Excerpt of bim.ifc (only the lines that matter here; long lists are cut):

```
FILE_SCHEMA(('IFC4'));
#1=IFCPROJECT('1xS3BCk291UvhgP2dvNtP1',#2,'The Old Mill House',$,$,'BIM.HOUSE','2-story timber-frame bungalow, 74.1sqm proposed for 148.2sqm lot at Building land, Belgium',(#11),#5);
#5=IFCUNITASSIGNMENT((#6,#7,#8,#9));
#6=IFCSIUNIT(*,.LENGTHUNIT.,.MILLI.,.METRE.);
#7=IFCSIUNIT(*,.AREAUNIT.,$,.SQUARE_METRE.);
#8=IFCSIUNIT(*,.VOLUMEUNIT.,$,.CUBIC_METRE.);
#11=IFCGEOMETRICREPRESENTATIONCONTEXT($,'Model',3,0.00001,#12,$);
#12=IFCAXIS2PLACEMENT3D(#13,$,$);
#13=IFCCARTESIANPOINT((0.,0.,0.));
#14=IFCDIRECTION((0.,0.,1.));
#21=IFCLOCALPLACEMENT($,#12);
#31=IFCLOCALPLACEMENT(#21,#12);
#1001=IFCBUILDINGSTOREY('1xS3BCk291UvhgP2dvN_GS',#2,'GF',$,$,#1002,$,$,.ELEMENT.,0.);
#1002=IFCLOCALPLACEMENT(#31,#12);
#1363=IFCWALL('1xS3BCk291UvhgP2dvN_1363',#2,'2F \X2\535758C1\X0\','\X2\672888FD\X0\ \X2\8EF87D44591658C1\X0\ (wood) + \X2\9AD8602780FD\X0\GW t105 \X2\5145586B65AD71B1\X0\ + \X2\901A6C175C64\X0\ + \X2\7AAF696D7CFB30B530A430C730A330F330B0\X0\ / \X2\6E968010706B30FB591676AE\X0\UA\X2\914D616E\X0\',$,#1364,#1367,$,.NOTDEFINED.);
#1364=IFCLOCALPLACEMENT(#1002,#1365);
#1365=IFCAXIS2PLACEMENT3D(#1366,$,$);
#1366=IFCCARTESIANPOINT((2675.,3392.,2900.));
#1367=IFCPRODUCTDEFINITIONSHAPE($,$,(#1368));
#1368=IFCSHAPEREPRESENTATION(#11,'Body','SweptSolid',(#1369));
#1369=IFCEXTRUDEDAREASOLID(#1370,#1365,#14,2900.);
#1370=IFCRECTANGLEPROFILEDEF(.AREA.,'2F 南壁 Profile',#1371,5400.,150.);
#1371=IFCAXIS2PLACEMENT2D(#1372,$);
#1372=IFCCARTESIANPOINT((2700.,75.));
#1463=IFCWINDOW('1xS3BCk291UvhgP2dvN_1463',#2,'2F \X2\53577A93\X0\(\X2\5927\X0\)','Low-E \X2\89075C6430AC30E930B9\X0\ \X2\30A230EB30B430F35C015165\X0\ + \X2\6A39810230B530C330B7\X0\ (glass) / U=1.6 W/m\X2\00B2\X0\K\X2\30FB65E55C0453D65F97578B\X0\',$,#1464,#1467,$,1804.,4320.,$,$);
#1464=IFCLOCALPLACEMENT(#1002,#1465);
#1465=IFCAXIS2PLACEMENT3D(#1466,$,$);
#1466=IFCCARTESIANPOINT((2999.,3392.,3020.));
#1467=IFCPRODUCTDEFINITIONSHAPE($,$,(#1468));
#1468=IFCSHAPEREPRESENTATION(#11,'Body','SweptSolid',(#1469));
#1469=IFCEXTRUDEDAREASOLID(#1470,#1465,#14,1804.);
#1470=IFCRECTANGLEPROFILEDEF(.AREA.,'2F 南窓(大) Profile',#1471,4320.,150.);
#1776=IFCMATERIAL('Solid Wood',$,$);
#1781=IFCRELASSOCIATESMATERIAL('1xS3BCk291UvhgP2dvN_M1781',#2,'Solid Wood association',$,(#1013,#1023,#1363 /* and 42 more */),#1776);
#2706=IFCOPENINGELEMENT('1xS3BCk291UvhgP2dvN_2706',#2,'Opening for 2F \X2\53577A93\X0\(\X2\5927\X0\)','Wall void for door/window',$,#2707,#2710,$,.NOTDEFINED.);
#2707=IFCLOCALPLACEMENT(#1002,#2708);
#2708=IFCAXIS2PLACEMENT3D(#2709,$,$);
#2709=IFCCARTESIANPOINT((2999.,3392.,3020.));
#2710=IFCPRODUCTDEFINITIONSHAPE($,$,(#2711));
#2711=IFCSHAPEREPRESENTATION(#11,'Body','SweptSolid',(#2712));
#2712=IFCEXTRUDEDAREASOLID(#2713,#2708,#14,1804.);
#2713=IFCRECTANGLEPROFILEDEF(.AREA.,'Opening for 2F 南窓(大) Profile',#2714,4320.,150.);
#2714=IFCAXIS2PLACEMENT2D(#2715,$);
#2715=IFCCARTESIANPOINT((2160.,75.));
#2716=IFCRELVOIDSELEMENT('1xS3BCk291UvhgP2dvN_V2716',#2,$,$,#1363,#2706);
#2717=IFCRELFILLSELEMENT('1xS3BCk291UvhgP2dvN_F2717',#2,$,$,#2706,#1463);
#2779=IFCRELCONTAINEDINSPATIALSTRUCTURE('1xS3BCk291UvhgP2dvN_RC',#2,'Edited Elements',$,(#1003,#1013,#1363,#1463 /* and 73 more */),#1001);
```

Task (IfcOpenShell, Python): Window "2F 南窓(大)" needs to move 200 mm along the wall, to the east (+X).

```python
import ifcopenshell
import ifcopenshell.api.geometry
import ifcopenshell.util.placement
import ifcopenshell.util.unit

model = ifcopenshell.open("bim.ifc")
unit_scale = ifcopenshell.util.unit.calculate_unit_scale(model)

window = model.by_id(1463)
opening = window.FillsVoids[0].RelatingOpeningElement
wall = opening.VoidsElements[0].RelatingBuildingElement

wall_matrix = ifcopenshell.util.placement.get_local_placement(wall.ObjectPlacement)
shift = wall_matrix[:3, 0] * 0.2 / unit_scale
before = ifcopenshell.util.placement.get_local_placement(window.ObjectPlacement)[:3, 3].copy()

# The window is not placed relative to its opening, so move both.
for product in (opening, window):
    matrix = ifcopenshell.util.placement.get_local_placement(product.ObjectPlacement)
    matrix[:3, 3] += shift
    ifcopenshell.api.geometry.edit_object_placement(model, product=product, matrix=matrix, is_si=False)

after = ifcopenshell.util.placement.get_local_placement(window.ObjectPlacement)[:3, 3]
print("window moved by", (after - before).round(3) + 0.0)

model.write("bim_edited.ifc")
```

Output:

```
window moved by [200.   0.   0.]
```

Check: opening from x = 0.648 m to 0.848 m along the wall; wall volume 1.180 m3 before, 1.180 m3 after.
